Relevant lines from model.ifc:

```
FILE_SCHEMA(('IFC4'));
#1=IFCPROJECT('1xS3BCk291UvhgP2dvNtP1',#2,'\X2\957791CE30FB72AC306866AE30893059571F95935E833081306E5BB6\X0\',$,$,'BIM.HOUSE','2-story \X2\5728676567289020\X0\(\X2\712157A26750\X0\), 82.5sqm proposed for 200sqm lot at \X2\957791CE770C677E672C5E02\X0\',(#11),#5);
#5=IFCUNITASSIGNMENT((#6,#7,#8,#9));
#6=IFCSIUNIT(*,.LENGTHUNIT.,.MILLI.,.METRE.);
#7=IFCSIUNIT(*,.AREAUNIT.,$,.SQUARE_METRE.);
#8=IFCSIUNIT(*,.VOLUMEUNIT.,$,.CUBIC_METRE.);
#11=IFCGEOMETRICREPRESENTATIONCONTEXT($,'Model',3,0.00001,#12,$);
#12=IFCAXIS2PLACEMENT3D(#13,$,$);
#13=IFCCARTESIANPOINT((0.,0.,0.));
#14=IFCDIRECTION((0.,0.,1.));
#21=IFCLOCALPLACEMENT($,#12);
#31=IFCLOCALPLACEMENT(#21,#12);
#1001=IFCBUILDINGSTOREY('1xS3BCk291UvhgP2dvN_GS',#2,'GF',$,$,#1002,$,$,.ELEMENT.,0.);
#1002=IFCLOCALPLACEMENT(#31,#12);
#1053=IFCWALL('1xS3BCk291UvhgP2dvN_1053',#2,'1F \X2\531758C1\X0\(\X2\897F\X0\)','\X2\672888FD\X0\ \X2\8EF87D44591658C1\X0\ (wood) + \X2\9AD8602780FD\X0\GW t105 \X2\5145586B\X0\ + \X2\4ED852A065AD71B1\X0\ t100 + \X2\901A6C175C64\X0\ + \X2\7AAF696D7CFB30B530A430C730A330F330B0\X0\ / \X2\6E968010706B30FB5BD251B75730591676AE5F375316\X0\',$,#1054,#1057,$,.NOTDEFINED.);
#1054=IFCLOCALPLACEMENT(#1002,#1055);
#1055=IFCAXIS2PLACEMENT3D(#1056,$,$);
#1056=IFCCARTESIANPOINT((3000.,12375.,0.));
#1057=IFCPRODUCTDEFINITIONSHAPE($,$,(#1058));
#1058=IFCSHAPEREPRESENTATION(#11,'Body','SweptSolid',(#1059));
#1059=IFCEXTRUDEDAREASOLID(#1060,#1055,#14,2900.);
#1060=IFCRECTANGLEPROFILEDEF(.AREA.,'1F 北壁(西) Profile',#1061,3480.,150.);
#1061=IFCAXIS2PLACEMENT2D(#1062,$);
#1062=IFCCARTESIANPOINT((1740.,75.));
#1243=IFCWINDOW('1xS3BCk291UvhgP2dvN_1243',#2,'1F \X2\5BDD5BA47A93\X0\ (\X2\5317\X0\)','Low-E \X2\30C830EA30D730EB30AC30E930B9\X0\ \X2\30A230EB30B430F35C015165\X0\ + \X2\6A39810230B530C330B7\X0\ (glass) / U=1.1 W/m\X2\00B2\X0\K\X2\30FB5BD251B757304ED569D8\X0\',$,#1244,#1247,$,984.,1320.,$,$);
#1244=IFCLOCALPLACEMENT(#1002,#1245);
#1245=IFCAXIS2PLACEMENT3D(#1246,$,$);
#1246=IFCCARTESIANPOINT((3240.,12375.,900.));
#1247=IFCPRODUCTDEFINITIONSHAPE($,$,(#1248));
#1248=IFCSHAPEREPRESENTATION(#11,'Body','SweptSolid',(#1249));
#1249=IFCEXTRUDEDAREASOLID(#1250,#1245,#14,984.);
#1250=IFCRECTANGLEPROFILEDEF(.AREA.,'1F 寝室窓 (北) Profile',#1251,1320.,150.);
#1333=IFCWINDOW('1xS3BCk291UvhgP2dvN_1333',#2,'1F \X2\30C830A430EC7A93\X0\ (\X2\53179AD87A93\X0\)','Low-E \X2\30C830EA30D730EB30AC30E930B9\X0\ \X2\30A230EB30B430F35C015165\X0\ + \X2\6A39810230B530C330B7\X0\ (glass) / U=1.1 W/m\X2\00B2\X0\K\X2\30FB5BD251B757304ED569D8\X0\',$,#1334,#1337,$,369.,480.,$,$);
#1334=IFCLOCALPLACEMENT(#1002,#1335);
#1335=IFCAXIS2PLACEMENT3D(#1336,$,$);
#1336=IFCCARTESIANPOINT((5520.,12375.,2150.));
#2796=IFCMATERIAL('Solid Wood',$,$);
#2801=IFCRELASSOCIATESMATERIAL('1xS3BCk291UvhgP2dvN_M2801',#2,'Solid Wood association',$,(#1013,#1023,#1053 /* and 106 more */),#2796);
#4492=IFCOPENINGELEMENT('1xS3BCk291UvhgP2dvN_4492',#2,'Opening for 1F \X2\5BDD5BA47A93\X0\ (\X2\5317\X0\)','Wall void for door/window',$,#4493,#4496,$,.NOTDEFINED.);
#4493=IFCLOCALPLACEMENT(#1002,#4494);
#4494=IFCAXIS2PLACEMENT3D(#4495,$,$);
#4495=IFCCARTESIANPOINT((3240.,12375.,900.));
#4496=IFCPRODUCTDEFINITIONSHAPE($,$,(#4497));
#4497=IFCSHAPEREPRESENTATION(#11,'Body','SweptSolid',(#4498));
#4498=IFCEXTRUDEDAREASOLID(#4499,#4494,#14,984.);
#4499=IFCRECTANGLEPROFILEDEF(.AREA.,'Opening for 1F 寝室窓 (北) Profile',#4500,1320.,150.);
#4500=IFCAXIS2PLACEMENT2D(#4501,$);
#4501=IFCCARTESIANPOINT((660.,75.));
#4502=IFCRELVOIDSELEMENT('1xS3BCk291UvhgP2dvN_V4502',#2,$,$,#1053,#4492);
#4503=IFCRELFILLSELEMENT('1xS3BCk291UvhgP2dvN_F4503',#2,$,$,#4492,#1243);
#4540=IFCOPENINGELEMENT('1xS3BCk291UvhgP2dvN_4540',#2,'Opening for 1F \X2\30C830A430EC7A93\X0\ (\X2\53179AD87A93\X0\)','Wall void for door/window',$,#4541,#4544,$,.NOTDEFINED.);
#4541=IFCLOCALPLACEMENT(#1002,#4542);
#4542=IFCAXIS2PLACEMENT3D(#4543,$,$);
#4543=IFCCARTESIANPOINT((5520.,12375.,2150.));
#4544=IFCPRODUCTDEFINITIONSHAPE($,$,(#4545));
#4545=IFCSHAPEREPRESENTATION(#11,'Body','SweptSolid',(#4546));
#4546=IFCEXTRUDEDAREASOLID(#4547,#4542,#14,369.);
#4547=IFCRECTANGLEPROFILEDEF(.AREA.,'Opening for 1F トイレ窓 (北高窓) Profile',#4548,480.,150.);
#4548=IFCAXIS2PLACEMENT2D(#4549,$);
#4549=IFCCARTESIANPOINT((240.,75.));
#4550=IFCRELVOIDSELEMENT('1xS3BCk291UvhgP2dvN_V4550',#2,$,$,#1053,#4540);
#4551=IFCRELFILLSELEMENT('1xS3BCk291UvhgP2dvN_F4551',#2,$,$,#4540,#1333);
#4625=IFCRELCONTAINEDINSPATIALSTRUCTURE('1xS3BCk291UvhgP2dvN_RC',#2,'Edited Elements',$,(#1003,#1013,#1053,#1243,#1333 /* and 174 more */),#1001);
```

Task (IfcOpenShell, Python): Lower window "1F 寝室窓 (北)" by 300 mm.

```python
import numpy as np
import ifcopenshell
import ifcopenshell.api.geometry
import ifcopenshell.util.placement
import ifcopenshell.util.unit

model = ifcopenshell.open("model.ifc")
unit_scale = ifcopenshell.util.unit.calculate_unit_scale(model)

window = model.by_guid("1xS3BCk291UvhgP2dvN_1243")
opening = window.FillsVoids[0].RelatingOpeningElement
dz = -300.0

shift = np.array([0.0, 0.0, dz])
# The window is not placed relative to its opening, so move both.
for product in (opening, window):
    matrix = ifcopenshell.util.placement.get_local_placement(product.ObjectPlacement)
    matrix[:3, 3] += shift
    ifcopenshell.api.geometry.edit_object_placement(model, product=product, matrix=matrix, is_si=False)

print(f"moved by {dz * unit_scale:+.3f} m")

model.write("model_v2.ifc")
```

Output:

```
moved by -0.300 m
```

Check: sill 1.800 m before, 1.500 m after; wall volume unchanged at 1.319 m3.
